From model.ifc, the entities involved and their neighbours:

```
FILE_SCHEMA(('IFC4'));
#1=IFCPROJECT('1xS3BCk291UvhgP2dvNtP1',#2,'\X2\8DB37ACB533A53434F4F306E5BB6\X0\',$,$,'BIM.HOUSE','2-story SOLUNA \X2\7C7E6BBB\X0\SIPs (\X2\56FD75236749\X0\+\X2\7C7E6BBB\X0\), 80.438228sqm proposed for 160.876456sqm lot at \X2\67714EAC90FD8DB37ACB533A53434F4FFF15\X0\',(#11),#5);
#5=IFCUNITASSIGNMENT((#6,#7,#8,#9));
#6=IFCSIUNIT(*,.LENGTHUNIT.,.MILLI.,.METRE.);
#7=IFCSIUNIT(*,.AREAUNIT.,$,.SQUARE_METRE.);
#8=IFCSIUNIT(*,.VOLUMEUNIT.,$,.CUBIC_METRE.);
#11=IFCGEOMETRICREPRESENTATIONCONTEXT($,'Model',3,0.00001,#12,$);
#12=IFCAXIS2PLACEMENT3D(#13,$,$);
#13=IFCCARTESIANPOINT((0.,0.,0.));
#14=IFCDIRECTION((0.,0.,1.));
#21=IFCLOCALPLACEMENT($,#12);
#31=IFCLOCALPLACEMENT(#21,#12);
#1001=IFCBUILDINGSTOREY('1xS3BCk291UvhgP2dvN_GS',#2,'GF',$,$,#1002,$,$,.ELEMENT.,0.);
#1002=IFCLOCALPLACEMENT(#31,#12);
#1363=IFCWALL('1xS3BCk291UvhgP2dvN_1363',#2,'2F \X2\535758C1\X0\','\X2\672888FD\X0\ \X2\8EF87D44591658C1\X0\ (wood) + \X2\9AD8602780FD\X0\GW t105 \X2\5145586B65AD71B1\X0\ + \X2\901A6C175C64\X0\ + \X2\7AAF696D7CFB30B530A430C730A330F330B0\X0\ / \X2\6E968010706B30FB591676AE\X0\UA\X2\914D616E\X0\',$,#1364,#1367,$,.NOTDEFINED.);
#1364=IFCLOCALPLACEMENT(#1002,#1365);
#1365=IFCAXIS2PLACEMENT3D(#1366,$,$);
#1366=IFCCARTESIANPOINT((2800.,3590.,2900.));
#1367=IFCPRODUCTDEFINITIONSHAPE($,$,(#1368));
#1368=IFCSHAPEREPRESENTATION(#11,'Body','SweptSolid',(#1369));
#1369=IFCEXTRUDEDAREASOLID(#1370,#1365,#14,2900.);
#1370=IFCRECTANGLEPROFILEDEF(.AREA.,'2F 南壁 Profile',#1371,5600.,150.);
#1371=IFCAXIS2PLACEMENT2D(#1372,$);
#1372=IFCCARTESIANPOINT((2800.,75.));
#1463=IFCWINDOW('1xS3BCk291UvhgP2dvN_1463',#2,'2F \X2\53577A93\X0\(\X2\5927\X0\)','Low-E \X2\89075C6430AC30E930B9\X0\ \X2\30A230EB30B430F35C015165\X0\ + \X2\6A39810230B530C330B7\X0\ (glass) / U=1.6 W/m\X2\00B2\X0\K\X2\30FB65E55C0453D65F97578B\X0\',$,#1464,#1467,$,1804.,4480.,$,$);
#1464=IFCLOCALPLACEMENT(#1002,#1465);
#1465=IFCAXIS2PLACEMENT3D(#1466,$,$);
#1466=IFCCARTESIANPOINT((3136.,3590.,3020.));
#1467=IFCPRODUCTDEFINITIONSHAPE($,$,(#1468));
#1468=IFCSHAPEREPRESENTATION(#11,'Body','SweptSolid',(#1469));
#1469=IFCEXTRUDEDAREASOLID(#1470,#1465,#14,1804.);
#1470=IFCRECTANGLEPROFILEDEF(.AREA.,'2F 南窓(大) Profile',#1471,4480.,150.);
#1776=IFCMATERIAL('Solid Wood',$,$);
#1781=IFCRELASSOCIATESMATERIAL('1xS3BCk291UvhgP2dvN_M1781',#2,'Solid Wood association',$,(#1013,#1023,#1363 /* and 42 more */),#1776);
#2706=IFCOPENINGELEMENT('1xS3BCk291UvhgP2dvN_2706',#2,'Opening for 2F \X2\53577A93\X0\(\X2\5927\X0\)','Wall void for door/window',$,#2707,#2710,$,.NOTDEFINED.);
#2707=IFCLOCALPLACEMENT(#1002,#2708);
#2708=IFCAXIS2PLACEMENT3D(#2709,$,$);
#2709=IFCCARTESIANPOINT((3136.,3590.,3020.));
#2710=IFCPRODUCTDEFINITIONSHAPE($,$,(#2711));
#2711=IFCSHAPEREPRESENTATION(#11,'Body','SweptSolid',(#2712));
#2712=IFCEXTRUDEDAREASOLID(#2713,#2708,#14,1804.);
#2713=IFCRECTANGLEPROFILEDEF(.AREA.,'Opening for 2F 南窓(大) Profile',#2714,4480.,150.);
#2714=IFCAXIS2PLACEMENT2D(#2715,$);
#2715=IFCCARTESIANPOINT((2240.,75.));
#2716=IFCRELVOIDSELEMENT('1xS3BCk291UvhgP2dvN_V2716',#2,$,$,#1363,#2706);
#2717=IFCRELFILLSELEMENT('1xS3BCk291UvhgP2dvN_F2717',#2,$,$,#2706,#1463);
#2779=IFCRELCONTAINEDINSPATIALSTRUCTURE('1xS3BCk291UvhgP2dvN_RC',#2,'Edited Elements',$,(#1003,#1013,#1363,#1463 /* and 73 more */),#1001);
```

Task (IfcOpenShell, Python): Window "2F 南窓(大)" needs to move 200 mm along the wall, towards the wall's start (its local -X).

```python
import ifcopenshell
import ifcopenshell.api.geometry
import ifcopenshell.util.placement

model = ifcopenshell.open("model.ifc")

window = model.by_id(1463)
opening = window.FillsVoids[0].RelatingOpeningElement
wall = opening.VoidsElements[0].RelatingBuildingElement

wall_matrix = ifcopenshell.util.placement.get_local_placement(wall.ObjectPlacement)
shift = wall_matrix[:3, 0] * -200.0
before = ifcopenshell.util.placement.get_local_placement(window.ObjectPlacement)[:3, 3].copy()

# The window is not placed relative to its opening, so move both.
for product in (opening, window):
    matrix = ifcopenshell.util.placement.get_local_placement(product.ObjectPlacement)
    matrix[:3, 3] += shift
    ifcopenshell.api.geometry.edit_object_placement(model, product=product, matrix=matrix, is_si=False)

after = ifcopenshell.util.placement.get_local_placement(window.ObjectPlacement)[:3, 3]
print("window moved by", (after - before).round(3) + 0.0)

model.write("model-out.ifc")
```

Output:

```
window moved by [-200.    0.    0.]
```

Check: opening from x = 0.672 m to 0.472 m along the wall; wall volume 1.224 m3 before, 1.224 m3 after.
